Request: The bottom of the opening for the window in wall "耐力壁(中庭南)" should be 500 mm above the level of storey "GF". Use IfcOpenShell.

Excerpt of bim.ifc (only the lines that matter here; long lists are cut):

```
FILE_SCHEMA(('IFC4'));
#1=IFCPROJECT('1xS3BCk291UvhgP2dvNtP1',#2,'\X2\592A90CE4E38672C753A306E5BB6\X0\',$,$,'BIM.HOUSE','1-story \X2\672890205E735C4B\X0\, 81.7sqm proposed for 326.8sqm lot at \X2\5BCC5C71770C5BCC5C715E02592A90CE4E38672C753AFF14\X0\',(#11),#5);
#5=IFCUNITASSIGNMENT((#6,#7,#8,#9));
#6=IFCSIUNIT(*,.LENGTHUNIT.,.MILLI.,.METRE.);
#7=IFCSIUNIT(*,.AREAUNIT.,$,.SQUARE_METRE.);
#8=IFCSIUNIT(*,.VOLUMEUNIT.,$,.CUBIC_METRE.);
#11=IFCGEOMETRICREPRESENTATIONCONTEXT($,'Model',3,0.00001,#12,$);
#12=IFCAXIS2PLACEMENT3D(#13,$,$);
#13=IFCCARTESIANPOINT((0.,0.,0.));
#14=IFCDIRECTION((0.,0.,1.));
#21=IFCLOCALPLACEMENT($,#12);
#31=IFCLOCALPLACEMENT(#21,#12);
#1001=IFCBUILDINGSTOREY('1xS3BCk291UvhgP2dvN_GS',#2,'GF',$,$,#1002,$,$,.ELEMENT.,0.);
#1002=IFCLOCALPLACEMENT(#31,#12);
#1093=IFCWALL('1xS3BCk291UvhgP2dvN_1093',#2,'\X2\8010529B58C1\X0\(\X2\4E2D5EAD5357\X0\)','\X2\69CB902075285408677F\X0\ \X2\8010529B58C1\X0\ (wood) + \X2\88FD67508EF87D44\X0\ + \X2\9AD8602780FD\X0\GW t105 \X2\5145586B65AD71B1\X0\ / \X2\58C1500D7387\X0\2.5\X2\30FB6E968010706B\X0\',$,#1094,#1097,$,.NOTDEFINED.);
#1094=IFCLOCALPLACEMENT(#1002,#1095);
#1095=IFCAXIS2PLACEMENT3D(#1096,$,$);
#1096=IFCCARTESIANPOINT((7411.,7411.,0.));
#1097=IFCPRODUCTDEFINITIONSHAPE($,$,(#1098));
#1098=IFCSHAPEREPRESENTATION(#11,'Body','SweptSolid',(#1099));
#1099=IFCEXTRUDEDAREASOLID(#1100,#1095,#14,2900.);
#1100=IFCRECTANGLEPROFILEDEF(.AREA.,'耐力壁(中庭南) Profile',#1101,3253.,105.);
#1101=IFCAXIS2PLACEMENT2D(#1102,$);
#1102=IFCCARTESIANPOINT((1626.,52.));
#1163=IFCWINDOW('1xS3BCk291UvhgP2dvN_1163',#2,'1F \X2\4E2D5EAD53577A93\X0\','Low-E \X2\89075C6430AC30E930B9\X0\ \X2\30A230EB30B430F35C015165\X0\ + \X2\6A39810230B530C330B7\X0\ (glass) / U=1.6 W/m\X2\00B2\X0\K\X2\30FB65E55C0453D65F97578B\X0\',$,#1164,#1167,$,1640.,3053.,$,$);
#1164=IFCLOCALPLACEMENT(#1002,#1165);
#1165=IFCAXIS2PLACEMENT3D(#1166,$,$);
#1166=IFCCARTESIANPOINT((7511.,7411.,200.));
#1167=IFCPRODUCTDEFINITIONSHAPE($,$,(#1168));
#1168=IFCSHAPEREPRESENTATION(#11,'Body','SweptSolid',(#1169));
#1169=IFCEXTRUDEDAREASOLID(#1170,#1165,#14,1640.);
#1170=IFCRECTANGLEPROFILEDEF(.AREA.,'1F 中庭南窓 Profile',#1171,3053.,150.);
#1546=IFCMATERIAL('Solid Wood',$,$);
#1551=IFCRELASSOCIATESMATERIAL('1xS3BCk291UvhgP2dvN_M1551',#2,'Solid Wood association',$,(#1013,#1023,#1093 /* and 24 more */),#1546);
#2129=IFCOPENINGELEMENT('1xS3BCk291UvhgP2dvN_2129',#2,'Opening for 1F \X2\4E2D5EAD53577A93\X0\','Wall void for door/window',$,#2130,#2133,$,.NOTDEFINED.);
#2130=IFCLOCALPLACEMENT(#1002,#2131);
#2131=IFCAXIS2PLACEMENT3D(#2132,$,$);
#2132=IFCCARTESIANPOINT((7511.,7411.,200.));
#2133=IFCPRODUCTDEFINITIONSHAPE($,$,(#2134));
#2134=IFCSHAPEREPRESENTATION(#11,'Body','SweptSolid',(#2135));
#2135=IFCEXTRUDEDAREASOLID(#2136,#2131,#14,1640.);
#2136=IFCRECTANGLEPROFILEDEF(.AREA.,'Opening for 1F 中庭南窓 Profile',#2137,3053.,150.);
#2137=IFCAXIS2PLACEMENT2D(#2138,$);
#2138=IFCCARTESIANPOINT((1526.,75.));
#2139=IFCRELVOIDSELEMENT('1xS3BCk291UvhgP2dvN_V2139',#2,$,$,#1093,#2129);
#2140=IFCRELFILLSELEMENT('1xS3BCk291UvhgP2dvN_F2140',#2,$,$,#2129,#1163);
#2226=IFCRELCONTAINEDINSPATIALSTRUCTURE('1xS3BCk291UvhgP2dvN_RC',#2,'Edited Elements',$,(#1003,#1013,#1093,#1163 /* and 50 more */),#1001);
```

```python
import numpy as np
import ifcopenshell
import ifcopenshell.api.geometry
import ifcopenshell.geom
import ifcopenshell.util.element
import ifcopenshell.util.placement
import ifcopenshell.util.shape
import ifcopenshell.util.unit

model = ifcopenshell.open("bim.ifc")
unit_scale = ifcopenshell.util.unit.calculate_unit_scale(model)

window = model.by_id(1163)
opening = window.FillsVoids[0].RelatingOpeningElement
storey = ifcopenshell.util.element.get_container(window, ifc_class="IfcBuildingStorey")
level = ifcopenshell.util.placement.get_local_placement(storey.ObjectPlacement)[2, 3]

# The opening's origin need not be at the sill, so measure its lowest point.
shape = ifcopenshell.geom.create_shape(ifcopenshell.geom.settings(), opening)
bottom = ifcopenshell.util.shape.get_shape_bottom_elevation(shape, shape.geometry) / unit_scale
dz = level + 500.0 - bottom

shift = np.array([0.0, 0.0, dz])
# The window is not placed relative to its opening, so move both.
for product in (opening, window):
    matrix = ifcopenshell.util.placement.get_local_placement(product.ObjectPlacement)
    matrix[:3, 3] += shift
    ifcopenshell.api.geometry.edit_object_placement(model, product=product, matrix=matrix, is_si=False)

print(f"moved by {dz * unit_scale:+.3f} m")

model.write("bim_rev.ifc")
```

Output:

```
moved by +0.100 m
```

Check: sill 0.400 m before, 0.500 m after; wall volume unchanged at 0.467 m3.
